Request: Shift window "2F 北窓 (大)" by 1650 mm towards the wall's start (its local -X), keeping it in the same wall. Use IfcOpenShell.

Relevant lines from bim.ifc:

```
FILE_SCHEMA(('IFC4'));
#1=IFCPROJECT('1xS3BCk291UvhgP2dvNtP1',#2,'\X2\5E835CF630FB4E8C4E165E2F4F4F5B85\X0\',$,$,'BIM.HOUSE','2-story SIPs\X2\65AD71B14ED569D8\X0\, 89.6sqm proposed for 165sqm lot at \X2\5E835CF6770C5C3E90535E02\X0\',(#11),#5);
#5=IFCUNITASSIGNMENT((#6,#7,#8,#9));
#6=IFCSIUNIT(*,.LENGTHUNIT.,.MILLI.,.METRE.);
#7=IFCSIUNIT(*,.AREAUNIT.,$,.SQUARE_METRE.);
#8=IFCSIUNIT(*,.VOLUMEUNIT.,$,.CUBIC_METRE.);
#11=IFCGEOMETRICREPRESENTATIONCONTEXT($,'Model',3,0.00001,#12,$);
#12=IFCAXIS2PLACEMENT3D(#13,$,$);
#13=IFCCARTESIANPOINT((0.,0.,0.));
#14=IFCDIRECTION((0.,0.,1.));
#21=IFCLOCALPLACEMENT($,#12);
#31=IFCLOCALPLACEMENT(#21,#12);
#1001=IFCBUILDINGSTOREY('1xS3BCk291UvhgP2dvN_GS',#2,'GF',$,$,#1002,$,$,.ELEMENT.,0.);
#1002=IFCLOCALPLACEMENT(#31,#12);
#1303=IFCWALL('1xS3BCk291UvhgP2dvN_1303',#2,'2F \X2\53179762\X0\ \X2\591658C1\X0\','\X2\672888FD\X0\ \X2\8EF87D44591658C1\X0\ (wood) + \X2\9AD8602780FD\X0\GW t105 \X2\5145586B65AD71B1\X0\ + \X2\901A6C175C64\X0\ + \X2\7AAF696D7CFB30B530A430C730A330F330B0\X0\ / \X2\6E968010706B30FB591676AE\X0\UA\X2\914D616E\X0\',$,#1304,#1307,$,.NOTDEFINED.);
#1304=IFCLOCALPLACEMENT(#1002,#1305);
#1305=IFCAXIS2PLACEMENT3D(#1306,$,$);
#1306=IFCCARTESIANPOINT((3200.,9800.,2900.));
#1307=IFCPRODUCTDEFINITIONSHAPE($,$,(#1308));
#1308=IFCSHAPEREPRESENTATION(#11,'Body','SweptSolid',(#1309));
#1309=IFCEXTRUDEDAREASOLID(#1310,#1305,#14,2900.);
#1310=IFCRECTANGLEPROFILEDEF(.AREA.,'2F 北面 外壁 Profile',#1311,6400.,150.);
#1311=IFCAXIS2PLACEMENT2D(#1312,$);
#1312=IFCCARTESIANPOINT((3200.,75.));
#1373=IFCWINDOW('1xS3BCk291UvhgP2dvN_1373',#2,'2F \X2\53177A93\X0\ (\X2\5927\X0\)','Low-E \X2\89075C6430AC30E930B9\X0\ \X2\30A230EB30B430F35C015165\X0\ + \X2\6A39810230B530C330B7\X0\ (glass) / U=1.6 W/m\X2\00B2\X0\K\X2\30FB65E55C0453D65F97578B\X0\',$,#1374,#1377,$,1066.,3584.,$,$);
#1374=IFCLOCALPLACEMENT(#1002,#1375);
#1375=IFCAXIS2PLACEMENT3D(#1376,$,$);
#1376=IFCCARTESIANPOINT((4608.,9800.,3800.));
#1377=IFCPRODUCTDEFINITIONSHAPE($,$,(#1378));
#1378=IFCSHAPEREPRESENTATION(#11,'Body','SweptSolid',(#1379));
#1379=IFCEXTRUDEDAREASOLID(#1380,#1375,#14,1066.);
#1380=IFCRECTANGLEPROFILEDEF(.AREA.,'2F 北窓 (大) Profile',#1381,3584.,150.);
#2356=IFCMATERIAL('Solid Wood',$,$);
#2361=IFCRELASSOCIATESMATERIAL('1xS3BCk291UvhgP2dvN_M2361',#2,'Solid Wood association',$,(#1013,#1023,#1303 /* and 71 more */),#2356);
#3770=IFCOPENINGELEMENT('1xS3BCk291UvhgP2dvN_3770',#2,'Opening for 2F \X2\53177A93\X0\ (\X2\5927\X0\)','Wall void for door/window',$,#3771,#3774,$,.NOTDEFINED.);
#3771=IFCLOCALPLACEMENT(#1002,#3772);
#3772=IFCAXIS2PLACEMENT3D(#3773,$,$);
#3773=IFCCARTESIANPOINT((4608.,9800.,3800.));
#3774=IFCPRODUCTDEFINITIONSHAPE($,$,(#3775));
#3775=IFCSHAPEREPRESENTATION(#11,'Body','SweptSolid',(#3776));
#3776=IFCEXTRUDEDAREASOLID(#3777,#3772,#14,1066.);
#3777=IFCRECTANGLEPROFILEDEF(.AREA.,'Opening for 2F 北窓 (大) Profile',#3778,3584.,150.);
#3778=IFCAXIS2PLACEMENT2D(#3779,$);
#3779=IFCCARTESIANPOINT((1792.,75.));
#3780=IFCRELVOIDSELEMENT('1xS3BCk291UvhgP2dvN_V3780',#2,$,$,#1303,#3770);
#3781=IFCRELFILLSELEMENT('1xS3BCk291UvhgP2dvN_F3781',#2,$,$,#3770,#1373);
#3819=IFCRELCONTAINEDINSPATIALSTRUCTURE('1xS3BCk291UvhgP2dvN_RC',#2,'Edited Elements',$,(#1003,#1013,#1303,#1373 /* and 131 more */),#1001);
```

```python
import ifcopenshell
import ifcopenshell.api.geometry
import ifcopenshell.util.placement

model = ifcopenshell.open("bim.ifc")

window = model.by_guid("1xS3BCk291UvhgP2dvN_1373")
opening = window.FillsVoids[0].RelatingOpeningElement
wall = opening.VoidsElements[0].RelatingBuildingElement

wall_matrix = ifcopenshell.util.placement.get_local_placement(wall.ObjectPlacement)
shift = wall_matrix[:3, 0] * -1650.0
before = ifcopenshell.util.placement.get_local_placement(window.ObjectPlacement)[:3, 3].copy()

# The window is not placed relative to its opening, so move both.
for product in (opening, window):
    matrix = ifcopenshell.util.placement.get_local_placement(product.ObjectPlacement)
    matrix[:3, 3] += shift
    ifcopenshell.api.geometry.edit_object_placement(model, product=product, matrix=matrix, is_si=False)

after = ifcopenshell.util.placement.get_local_placement(window.ObjectPlacement)[:3, 3]
print("window moved by", (after - before).round(3) + 0.0)

model.write("bim_v2.ifc")
```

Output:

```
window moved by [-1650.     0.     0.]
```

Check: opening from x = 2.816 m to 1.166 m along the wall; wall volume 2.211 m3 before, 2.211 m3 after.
